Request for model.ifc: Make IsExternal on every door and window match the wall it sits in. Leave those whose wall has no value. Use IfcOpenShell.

First a look at what the model holds.

```python
import ifcopenshell
import ifcopenshell.util.element

model = ifcopenshell.open("model.ifc")
print(model.schema)
seen = {}
for e in model.by_type("IfcDoor") + model.by_type("IfcWindow"):
    if not e.FillsVoids:
        continue
    host = e.FillsVoids[0].RelatingOpeningElement.VoidsElements[0].RelatingBuildingElement
    own = ifcopenshell.util.element.get_pset(e, f"Pset_{e.is_a()[3:].removesuffix('StandardCase')}Common", "IsExternal")
    wall = ifcopenshell.util.element.get_pset(host, "Pset_WallCommon", "IsExternal")
    seen[e.is_a(), own, wall] = seen.get((e.is_a(), own, wall), 0) + 1
for (cls, own, wall), count in sorted(seen.items(), key=str):
    print(count, cls, "IsExternal:", own, "| host wall:", wall)
```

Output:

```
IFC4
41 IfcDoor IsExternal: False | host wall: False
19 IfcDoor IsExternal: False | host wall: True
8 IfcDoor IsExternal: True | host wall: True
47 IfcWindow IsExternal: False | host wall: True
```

```python
import ifcopenshell
import ifcopenshell.api.pset
import ifcopenshell.util.element

model = ifcopenshell.open("model.ifc")

count = 0
for ifc_class, pset_name in (("IfcDoor", "Pset_DoorCommon"), ("IfcWindow", "Pset_WindowCommon")):
    for e in model.by_type(ifc_class):
        if not e.FillsVoids:
            continue
        host = e.FillsVoids[0].RelatingOpeningElement.VoidsElements[0].RelatingBuildingElement
        external = ifcopenshell.util.element.get_pset(host, "Pset_WallCommon", "IsExternal")
        if external is None or ifcopenshell.util.element.get_pset(e, pset_name, "IsExternal") == external:
            continue
        pset = ifcopenshell.api.pset.add_pset(model, product=e, name=pset_name)
        ifcopenshell.api.pset.edit_pset(model, pset=pset, properties={"IsExternal": external})
        count += 1

print(count, "updated")

model.write("model_updated.ifc")
```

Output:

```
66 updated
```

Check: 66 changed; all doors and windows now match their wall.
